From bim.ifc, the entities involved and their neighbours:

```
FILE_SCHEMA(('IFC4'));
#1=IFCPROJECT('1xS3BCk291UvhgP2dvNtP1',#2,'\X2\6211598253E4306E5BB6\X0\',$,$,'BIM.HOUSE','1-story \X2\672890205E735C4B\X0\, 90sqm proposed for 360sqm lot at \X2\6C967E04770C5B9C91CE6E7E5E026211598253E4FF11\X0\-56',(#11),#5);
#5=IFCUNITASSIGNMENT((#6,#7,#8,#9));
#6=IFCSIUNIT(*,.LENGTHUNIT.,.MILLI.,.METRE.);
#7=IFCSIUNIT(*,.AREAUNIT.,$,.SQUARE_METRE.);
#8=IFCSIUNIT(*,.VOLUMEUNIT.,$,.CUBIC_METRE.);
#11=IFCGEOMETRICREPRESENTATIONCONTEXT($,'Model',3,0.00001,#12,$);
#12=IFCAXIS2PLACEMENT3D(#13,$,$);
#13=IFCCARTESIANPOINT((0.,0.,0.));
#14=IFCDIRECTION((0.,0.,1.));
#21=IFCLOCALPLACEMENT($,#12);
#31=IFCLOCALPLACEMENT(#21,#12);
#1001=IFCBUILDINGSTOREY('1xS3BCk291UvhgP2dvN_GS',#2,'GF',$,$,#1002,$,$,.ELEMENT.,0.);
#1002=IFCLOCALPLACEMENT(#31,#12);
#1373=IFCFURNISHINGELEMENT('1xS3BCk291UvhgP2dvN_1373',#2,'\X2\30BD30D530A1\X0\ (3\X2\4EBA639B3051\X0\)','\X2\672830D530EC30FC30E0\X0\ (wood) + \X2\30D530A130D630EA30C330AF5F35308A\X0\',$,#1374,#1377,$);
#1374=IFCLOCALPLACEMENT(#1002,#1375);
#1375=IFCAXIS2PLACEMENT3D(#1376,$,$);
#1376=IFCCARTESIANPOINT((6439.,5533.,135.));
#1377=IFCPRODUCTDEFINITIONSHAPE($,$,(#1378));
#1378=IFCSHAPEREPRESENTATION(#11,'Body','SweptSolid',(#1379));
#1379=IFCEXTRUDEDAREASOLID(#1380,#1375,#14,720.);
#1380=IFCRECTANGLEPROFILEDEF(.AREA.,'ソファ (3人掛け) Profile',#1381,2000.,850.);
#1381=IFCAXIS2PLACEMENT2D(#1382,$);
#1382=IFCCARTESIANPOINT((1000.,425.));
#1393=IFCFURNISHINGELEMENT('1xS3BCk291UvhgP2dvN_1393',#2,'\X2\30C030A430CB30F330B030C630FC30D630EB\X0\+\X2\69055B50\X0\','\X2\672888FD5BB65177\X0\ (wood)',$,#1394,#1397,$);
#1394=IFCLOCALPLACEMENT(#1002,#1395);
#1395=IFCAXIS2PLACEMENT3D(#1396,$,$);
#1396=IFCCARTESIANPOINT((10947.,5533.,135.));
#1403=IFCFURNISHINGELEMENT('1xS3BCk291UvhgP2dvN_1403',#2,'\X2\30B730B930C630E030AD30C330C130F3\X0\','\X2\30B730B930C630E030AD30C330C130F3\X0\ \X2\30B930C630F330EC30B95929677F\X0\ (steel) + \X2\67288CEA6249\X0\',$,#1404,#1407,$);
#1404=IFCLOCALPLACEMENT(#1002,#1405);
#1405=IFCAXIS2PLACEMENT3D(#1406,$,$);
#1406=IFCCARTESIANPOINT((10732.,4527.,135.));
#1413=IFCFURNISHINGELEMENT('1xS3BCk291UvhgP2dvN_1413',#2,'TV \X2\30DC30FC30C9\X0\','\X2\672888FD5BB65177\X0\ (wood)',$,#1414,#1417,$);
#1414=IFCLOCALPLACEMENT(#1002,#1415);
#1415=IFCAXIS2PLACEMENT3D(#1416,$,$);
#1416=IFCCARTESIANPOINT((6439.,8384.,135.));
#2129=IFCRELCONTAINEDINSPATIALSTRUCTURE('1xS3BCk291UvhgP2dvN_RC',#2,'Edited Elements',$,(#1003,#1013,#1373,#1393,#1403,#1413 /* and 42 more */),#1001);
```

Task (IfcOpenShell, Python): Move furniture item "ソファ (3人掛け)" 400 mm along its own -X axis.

```python
import ifcopenshell
import ifcopenshell.api.geometry
import ifcopenshell.util.placement

model = ifcopenshell.open("bim.ifc")

item = model.by_guid("1xS3BCk291UvhgP2dvN_1373")
matrix = ifcopenshell.util.placement.get_local_placement(item.ObjectPlacement)
matrix[:3, 3] -= matrix[:3, 0] * 400.0
ifcopenshell.api.geometry.edit_object_placement(model, product=item, matrix=matrix, is_si=False)

print(ifcopenshell.util.placement.get_local_placement(item.ObjectPlacement).round(3) + 0.0)

model.write("bim_rev.ifc")
```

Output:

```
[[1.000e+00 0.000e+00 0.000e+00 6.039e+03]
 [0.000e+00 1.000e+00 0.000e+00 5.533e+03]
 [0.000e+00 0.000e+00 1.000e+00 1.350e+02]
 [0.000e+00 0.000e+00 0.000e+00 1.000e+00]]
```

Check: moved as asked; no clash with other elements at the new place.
